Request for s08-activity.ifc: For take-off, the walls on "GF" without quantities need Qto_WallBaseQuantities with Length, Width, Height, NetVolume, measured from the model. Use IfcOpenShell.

First a look at what the model holds.

```python
import ifcopenshell
import ifcopenshell.util.element
import ifcopenshell.util.unit

model = ifcopenshell.open("s08-activity.ifc")
print(model.schema)
for unit_type in ("LENGTHUNIT", "AREAUNIT", "VOLUMEUNIT"):
    print(unit_type, ifcopenshell.util.unit.calculate_unit_scale(model, unit_type))
storey = next(s for s in model.by_type("IfcBuildingStorey") if s.Name == "GF")
walls = [e for e in ifcopenshell.util.element.get_decomposition(storey) if e.is_a("IfcWall")]
for e in sorted(walls, key=lambda e: e.id()):
    print(e.id(), e.is_a(), e.Name, list(ifcopenshell.util.element.get_psets(e, qtos_only=True)), sep=" | ")
```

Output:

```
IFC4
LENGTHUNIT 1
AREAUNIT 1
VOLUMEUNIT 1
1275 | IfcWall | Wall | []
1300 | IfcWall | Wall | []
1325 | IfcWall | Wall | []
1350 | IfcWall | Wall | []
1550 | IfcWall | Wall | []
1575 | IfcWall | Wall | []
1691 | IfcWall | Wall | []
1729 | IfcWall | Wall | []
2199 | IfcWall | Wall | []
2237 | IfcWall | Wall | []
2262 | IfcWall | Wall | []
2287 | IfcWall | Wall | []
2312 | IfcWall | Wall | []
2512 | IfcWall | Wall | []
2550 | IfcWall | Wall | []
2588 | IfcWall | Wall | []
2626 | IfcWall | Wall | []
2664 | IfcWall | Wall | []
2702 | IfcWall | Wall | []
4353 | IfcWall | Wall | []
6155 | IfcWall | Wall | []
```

```python
import ifcopenshell
import ifcopenshell.api.pset
import ifcopenshell.geom
import ifcopenshell.util.element
import ifcopenshell.util.shape
import ifcopenshell.util.unit

model = ifcopenshell.open("s08-activity.ifc")
unit_scale = ifcopenshell.util.unit.calculate_unit_scale(model)
volume_scale = ifcopenshell.util.unit.calculate_unit_scale(model, "VOLUMEUNIT")
settings = ifcopenshell.geom.settings()

storey = next(s for s in model.by_type("IfcBuildingStorey") if s.Name == "GF")
walls = [e for e in ifcopenshell.util.element.get_decomposition(storey) if e.is_a("IfcWall")]

for e in sorted(walls, key=lambda e: e.id()):
    if ifcopenshell.util.element.get_psets(e, qtos_only=True, should_inherit=False):
        continue
    # Geometry comes back in metres, in the element's own axes.
    shape = ifcopenshell.geom.create_shape(settings, e)
    values = {
        "Length": ifcopenshell.util.shape.get_x(shape.geometry) / unit_scale,
        "Width": ifcopenshell.util.shape.get_y(shape.geometry) / unit_scale,
        "Height": ifcopenshell.util.shape.get_z(shape.geometry) / unit_scale,
        "NetVolume": ifcopenshell.util.shape.get_volume(shape.geometry) / volume_scale,
    }
    qto = ifcopenshell.api.pset.add_qto(model, product=e, name="Qto_WallBaseQuantities")
    ifcopenshell.api.pset.edit_qto(model, qto=qto, properties=values)
    print(e.id(), {k: round(v, 3) for k, v in values.items()})

model.write("s08-activity_rev.ifc")
```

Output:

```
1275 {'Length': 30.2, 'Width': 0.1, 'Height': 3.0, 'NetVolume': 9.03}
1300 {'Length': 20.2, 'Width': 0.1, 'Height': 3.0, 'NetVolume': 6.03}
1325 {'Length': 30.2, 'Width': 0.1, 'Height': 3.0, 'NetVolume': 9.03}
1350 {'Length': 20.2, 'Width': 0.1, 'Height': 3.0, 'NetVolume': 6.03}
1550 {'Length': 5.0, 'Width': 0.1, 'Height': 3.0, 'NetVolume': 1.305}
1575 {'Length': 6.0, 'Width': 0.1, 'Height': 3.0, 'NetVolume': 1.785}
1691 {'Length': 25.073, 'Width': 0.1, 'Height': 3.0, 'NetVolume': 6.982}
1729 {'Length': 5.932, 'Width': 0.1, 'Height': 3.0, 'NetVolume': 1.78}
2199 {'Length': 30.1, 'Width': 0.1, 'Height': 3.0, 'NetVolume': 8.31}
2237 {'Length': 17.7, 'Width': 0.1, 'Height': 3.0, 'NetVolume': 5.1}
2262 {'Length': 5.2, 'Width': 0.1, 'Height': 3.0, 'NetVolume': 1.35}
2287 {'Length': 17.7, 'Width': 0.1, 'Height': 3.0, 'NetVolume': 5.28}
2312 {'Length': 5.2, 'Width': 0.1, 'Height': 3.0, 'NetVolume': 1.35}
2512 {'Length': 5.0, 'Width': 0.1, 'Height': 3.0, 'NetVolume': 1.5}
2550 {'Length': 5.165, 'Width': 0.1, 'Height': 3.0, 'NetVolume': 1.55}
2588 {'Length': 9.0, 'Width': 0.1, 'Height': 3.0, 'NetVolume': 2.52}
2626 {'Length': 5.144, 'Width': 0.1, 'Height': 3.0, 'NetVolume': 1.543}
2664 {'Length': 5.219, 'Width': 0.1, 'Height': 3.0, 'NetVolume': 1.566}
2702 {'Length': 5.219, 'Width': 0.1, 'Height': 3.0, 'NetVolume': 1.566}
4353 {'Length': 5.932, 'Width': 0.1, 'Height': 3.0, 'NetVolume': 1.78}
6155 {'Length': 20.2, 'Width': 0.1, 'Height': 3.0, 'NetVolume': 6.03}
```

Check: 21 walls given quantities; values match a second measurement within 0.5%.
